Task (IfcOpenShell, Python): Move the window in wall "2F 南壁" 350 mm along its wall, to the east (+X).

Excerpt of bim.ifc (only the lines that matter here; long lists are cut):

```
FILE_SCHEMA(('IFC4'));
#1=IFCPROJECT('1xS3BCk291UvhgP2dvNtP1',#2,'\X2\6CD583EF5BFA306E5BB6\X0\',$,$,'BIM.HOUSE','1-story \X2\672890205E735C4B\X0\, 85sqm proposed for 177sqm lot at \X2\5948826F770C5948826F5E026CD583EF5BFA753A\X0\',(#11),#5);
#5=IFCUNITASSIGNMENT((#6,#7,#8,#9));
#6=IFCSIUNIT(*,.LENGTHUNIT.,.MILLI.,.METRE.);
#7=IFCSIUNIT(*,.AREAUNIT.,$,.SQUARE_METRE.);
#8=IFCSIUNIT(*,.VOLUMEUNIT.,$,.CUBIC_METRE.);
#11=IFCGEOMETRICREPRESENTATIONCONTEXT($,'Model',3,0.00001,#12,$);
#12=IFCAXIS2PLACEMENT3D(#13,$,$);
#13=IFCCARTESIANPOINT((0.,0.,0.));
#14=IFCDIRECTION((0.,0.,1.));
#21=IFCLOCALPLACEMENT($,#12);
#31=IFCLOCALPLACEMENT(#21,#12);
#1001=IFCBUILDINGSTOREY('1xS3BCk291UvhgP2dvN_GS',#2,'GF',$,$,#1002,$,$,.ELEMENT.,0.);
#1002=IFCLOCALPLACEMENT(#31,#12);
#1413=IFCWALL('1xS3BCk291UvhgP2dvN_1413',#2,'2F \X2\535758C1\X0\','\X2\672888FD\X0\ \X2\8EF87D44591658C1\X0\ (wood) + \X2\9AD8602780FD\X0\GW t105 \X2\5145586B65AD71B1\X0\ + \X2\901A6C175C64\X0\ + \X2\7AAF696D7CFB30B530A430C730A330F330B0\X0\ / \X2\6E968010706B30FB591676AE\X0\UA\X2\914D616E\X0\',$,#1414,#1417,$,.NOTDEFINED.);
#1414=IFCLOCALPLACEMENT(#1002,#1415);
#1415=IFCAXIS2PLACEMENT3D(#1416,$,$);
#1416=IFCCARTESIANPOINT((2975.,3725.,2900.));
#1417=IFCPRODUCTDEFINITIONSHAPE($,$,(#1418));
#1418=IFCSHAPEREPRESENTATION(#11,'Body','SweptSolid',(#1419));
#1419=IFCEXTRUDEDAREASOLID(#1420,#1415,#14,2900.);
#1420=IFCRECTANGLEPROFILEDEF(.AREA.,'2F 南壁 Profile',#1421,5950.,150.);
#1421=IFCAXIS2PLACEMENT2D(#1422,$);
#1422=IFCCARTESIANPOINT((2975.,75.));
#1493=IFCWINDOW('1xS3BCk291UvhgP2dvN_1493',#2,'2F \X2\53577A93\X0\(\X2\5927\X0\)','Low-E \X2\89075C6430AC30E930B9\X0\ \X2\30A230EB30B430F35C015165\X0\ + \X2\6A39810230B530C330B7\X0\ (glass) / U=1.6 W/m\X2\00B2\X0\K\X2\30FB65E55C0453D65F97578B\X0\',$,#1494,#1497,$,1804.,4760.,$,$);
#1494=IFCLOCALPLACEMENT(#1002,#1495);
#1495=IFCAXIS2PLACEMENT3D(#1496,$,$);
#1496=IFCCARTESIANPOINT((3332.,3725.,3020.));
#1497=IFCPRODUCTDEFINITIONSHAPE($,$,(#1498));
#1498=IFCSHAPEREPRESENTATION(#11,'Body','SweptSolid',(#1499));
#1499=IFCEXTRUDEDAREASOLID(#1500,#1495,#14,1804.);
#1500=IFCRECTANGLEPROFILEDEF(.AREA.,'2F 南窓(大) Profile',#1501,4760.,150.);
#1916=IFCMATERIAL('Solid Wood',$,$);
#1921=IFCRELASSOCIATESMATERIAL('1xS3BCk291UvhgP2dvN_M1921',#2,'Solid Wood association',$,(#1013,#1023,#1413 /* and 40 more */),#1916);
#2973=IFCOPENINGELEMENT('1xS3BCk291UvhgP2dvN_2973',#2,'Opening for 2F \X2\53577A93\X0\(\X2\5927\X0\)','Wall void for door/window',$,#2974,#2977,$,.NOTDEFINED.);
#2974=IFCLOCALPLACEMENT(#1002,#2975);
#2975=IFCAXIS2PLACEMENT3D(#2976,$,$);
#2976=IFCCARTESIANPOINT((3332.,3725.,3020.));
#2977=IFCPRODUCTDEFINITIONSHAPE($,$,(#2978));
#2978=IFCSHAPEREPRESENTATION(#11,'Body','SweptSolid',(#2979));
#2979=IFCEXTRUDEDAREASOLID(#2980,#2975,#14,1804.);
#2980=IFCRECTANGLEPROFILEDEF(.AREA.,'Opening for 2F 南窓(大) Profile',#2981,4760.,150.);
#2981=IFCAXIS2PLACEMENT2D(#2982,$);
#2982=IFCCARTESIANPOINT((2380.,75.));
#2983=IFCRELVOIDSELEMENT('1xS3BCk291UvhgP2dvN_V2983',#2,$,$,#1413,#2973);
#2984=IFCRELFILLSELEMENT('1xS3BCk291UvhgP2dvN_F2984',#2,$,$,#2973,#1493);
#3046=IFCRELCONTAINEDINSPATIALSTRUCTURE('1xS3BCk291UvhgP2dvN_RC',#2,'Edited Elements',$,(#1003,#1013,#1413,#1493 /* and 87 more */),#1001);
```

```python
import ifcopenshell
import ifcopenshell.api.geometry
import ifcopenshell.util.placement
import ifcopenshell.util.unit

model = ifcopenshell.open("bim.ifc")
unit_scale = ifcopenshell.util.unit.calculate_unit_scale(model)

window = model.by_guid("1xS3BCk291UvhgP2dvN_1493")
opening = window.FillsVoids[0].RelatingOpeningElement
wall = opening.VoidsElements[0].RelatingBuildingElement

wall_matrix = ifcopenshell.util.placement.get_local_placement(wall.ObjectPlacement)
shift = wall_matrix[:3, 0] * 0.35 / unit_scale
before = ifcopenshell.util.placement.get_local_placement(window.ObjectPlacement)[:3, 3].copy()

# The window is not placed relative to its opening, so move both.
for product in (opening, window):
    matrix = ifcopenshell.util.placement.get_local_placement(product.ObjectPlacement)
    matrix[:3, 3] += shift
    ifcopenshell.api.geometry.edit_object_placement(model, product=product, matrix=matrix, is_si=False)

after = ifcopenshell.util.placement.get_local_placement(window.ObjectPlacement)[:3, 3]
print("window moved by", (after - before).round(3) + 0.0)

model.write("bim_edited.ifc")
```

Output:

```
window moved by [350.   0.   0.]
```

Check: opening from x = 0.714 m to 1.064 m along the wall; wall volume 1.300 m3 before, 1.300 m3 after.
